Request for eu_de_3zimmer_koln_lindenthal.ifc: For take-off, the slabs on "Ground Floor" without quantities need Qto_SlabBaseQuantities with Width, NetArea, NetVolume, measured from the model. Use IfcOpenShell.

First a look at what the model holds.

```python
import ifcopenshell
import ifcopenshell.util.element
import ifcopenshell.util.unit

model = ifcopenshell.open("eu_de_3zimmer_koln_lindenthal.ifc")
print(model.schema)
for unit_type in ("LENGTHUNIT", "AREAUNIT", "VOLUMEUNIT"):
    print(unit_type, ifcopenshell.util.unit.calculate_unit_scale(model, unit_type))
storey = next(s for s in model.by_type("IfcBuildingStorey") if s.Name == "Ground Floor")
slabs = [e for e in ifcopenshell.util.element.get_decomposition(storey) if e.is_a("IfcSlab")]
for e in sorted(slabs, key=lambda e: e.id()):
    print(e.id(), e.is_a(), e.Name, list(ifcopenshell.util.element.get_psets(e, qtos_only=True)), sep=" | ")
```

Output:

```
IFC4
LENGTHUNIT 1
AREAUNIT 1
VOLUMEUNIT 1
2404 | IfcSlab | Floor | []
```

```python
import ifcopenshell
import ifcopenshell.api.pset
import ifcopenshell.geom
import ifcopenshell.util.element
import ifcopenshell.util.shape
import ifcopenshell.util.unit

model = ifcopenshell.open("eu_de_3zimmer_koln_lindenthal.ifc")
unit_scale = ifcopenshell.util.unit.calculate_unit_scale(model)
area_scale = ifcopenshell.util.unit.calculate_unit_scale(model, "AREAUNIT")
volume_scale = ifcopenshell.util.unit.calculate_unit_scale(model, "VOLUMEUNIT")
settings = ifcopenshell.geom.settings()

storey = next(s for s in model.by_type("IfcBuildingStorey") if s.Name == "Ground Floor")
slabs = [e for e in ifcopenshell.util.element.get_decomposition(storey) if e.is_a("IfcSlab")]

for e in sorted(slabs, key=lambda e: e.id()):
    if ifcopenshell.util.element.get_psets(e, qtos_only=True, should_inherit=False):
        continue
    # Geometry comes back in metres, in the element's own axes.
    shape = ifcopenshell.geom.create_shape(settings, e)
    values = {
        "Width": ifcopenshell.util.shape.get_z(shape.geometry) / unit_scale,
        "NetArea": ifcopenshell.util.shape.get_footprint_area(shape.geometry) / area_scale,
        "NetVolume": ifcopenshell.util.shape.get_volume(shape.geometry) / volume_scale,
    }
    qto = ifcopenshell.api.pset.add_qto(model, product=e, name="Qto_SlabBaseQuantities")
    ifcopenshell.api.pset.edit_qto(model, qto=qto, properties=values)
    print(e.id(), {k: round(v, 3) for k, v in values.items()})

model.write("eu_de_3zimmer_koln_lindenthal_edited.ifc")
```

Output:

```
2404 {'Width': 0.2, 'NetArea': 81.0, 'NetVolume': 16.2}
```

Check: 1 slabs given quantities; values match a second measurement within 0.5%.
